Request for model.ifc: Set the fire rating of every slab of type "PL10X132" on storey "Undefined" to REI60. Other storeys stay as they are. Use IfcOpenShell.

First a look at what the model holds.

```python
import ifcopenshell
import ifcopenshell.util.element

model = ifcopenshell.open("model.ifc")
print(model.schema)
storey = next(s for s in model.by_type("IfcBuildingStorey") if s.Name == "Undefined")
slabs = [e for e in ifcopenshell.util.element.get_decomposition(storey) if e.is_a("IfcSlab")]
seen = {}
for e in slabs:
    element_type = ifcopenshell.util.element.get_type(e)
    key = (element_type.Name if element_type != e and element_type else None, ifcopenshell.util.element.get_pset(e, "Pset_SlabCommon", "FireRating"))
    seen[key] = seen.get(key, 0) + 1
for (name, value), count in sorted(seen.items(), key=str):
    print(count, "x", name, "|", value)
```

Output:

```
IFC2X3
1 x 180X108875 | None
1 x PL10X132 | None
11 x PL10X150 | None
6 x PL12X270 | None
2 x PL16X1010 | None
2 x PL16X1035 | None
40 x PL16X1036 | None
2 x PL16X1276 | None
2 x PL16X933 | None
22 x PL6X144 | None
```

```python
import ifcopenshell
import ifcopenshell.api.pset
import ifcopenshell.util.element

model = ifcopenshell.open("model.ifc")

storey = next(s for s in model.by_type("IfcBuildingStorey") if s.Name == "Undefined")
slabs = [e for e in ifcopenshell.util.element.get_decomposition(storey) if e.is_a("IfcSlab")]

count = 0
for e in slabs:
    element_type = ifcopenshell.util.element.get_type(e)
    if element_type in (None, e) or element_type.Name != "PL10X132":
        continue
    # add_pset returns the element's existing set when there is one.
    pset = ifcopenshell.api.pset.add_pset(model, product=e, name="Pset_SlabCommon")
    ifcopenshell.api.pset.edit_pset(model, pset=pset, properties={"FireRating": "REI60"})
    count += 1

print(count, "slabs updated")

model.write("model_updated.ifc")
```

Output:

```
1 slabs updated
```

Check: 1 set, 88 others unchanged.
